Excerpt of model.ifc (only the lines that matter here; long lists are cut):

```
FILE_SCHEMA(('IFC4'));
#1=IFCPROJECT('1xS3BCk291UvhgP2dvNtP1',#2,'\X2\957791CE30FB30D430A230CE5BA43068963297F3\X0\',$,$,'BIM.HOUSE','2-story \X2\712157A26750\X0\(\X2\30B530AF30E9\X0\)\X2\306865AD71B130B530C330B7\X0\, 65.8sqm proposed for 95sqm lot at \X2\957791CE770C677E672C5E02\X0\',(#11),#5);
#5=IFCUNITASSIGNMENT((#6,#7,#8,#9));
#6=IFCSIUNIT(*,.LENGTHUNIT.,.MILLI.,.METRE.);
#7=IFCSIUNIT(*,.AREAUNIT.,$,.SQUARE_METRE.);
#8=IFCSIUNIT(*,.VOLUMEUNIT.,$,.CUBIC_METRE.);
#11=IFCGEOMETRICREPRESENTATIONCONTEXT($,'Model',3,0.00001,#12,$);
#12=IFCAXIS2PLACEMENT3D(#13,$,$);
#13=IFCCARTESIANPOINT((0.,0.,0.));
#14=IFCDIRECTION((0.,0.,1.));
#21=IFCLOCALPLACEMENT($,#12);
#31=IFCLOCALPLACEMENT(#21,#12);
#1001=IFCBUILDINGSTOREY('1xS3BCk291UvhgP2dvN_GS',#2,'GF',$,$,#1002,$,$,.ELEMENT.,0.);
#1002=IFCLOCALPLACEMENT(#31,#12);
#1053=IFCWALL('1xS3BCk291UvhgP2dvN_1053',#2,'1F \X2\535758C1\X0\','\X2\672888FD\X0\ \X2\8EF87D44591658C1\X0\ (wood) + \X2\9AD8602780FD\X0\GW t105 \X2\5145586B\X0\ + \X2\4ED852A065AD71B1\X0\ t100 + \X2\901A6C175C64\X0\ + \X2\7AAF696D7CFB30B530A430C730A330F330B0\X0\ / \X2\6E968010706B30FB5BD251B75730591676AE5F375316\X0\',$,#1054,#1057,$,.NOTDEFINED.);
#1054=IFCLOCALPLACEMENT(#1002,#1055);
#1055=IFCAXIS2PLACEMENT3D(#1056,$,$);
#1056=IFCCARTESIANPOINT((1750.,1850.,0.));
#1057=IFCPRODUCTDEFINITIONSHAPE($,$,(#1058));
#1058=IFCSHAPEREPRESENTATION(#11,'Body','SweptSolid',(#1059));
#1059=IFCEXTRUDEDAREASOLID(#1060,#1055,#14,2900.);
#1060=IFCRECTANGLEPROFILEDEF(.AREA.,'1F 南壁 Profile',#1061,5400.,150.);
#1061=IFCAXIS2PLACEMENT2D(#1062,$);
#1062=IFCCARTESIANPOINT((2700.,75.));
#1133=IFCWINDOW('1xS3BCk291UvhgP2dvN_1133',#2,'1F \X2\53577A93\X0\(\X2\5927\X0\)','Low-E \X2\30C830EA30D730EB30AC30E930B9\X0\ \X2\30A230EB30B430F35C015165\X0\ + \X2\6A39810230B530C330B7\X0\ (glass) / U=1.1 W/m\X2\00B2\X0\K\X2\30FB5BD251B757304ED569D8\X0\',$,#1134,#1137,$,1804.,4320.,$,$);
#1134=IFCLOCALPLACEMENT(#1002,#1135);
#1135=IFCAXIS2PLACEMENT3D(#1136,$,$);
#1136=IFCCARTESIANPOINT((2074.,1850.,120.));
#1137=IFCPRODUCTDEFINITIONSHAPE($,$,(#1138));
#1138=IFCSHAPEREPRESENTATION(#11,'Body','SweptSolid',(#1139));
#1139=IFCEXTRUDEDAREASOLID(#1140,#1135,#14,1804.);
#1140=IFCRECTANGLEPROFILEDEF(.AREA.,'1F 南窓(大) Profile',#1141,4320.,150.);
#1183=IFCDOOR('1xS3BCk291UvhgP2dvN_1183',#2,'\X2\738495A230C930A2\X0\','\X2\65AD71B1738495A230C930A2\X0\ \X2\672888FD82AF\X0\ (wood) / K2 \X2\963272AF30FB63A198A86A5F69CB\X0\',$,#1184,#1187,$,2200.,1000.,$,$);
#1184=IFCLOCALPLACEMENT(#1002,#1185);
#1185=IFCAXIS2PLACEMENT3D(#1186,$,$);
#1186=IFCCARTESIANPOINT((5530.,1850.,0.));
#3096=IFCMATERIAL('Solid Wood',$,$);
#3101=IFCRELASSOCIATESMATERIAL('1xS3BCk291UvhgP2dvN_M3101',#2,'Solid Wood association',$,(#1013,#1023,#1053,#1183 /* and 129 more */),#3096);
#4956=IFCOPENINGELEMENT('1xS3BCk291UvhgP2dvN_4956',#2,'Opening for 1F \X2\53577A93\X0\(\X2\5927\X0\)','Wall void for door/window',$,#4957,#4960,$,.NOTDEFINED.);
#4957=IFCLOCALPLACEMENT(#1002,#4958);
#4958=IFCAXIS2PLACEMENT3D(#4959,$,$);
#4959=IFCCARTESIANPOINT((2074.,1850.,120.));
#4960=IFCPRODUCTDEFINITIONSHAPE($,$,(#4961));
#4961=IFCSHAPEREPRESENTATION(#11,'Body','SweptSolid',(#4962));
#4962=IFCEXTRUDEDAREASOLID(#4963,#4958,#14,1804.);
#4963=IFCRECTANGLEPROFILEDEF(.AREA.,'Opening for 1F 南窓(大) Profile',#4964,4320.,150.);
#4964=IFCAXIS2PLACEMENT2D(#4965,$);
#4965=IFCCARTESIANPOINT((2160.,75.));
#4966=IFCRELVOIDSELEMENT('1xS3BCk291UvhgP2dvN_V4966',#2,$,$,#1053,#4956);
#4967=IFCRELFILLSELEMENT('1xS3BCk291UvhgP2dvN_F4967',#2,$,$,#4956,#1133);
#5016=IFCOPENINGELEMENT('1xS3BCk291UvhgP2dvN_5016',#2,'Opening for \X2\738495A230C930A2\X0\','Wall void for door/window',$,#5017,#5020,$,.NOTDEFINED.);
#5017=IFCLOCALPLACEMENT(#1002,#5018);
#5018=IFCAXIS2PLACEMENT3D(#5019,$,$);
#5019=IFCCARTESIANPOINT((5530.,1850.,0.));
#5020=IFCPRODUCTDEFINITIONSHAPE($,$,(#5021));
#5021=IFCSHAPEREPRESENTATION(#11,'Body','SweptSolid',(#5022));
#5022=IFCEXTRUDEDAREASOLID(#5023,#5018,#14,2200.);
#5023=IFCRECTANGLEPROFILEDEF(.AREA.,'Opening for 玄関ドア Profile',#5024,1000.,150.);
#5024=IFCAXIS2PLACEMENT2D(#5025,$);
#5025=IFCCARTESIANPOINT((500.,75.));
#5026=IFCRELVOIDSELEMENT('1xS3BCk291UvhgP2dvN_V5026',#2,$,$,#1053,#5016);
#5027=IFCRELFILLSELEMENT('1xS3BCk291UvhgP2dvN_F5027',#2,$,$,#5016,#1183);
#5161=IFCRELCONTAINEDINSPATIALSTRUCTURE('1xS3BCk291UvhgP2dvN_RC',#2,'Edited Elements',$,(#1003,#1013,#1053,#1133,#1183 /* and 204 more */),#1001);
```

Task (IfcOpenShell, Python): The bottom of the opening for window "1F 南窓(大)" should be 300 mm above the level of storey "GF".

```python
import numpy as np
import ifcopenshell
import ifcopenshell.api.geometry
import ifcopenshell.geom
import ifcopenshell.util.element
import ifcopenshell.util.placement
import ifcopenshell.util.shape
import ifcopenshell.util.unit

model = ifcopenshell.open("model.ifc")
unit_scale = ifcopenshell.util.unit.calculate_unit_scale(model)

window = model.by_id(1133)
opening = window.FillsVoids[0].RelatingOpeningElement
storey = ifcopenshell.util.element.get_container(window, ifc_class="IfcBuildingStorey")
level = ifcopenshell.util.placement.get_local_placement(storey.ObjectPlacement)[2, 3]

# The opening's origin need not be at the sill, so measure its lowest point.
shape = ifcopenshell.geom.create_shape(ifcopenshell.geom.settings(), opening)
bottom = ifcopenshell.util.shape.get_shape_bottom_elevation(shape, shape.geometry) / unit_scale
dz = level + 0.3 / unit_scale - bottom

shift = np.array([0.0, 0.0, dz])
# The window is not placed relative to its opening, so move both.
for product in (opening, window):
    matrix = ifcopenshell.util.placement.get_local_placement(product.ObjectPlacement)
    matrix[:3, 3] += shift
    ifcopenshell.api.geometry.edit_object_placement(model, product=product, matrix=matrix, is_si=False)

print(f"moved by {dz * unit_scale:+.3f} m")

model.write("model_updated.ifc")
```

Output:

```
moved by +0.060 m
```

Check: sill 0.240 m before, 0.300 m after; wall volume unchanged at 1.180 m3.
